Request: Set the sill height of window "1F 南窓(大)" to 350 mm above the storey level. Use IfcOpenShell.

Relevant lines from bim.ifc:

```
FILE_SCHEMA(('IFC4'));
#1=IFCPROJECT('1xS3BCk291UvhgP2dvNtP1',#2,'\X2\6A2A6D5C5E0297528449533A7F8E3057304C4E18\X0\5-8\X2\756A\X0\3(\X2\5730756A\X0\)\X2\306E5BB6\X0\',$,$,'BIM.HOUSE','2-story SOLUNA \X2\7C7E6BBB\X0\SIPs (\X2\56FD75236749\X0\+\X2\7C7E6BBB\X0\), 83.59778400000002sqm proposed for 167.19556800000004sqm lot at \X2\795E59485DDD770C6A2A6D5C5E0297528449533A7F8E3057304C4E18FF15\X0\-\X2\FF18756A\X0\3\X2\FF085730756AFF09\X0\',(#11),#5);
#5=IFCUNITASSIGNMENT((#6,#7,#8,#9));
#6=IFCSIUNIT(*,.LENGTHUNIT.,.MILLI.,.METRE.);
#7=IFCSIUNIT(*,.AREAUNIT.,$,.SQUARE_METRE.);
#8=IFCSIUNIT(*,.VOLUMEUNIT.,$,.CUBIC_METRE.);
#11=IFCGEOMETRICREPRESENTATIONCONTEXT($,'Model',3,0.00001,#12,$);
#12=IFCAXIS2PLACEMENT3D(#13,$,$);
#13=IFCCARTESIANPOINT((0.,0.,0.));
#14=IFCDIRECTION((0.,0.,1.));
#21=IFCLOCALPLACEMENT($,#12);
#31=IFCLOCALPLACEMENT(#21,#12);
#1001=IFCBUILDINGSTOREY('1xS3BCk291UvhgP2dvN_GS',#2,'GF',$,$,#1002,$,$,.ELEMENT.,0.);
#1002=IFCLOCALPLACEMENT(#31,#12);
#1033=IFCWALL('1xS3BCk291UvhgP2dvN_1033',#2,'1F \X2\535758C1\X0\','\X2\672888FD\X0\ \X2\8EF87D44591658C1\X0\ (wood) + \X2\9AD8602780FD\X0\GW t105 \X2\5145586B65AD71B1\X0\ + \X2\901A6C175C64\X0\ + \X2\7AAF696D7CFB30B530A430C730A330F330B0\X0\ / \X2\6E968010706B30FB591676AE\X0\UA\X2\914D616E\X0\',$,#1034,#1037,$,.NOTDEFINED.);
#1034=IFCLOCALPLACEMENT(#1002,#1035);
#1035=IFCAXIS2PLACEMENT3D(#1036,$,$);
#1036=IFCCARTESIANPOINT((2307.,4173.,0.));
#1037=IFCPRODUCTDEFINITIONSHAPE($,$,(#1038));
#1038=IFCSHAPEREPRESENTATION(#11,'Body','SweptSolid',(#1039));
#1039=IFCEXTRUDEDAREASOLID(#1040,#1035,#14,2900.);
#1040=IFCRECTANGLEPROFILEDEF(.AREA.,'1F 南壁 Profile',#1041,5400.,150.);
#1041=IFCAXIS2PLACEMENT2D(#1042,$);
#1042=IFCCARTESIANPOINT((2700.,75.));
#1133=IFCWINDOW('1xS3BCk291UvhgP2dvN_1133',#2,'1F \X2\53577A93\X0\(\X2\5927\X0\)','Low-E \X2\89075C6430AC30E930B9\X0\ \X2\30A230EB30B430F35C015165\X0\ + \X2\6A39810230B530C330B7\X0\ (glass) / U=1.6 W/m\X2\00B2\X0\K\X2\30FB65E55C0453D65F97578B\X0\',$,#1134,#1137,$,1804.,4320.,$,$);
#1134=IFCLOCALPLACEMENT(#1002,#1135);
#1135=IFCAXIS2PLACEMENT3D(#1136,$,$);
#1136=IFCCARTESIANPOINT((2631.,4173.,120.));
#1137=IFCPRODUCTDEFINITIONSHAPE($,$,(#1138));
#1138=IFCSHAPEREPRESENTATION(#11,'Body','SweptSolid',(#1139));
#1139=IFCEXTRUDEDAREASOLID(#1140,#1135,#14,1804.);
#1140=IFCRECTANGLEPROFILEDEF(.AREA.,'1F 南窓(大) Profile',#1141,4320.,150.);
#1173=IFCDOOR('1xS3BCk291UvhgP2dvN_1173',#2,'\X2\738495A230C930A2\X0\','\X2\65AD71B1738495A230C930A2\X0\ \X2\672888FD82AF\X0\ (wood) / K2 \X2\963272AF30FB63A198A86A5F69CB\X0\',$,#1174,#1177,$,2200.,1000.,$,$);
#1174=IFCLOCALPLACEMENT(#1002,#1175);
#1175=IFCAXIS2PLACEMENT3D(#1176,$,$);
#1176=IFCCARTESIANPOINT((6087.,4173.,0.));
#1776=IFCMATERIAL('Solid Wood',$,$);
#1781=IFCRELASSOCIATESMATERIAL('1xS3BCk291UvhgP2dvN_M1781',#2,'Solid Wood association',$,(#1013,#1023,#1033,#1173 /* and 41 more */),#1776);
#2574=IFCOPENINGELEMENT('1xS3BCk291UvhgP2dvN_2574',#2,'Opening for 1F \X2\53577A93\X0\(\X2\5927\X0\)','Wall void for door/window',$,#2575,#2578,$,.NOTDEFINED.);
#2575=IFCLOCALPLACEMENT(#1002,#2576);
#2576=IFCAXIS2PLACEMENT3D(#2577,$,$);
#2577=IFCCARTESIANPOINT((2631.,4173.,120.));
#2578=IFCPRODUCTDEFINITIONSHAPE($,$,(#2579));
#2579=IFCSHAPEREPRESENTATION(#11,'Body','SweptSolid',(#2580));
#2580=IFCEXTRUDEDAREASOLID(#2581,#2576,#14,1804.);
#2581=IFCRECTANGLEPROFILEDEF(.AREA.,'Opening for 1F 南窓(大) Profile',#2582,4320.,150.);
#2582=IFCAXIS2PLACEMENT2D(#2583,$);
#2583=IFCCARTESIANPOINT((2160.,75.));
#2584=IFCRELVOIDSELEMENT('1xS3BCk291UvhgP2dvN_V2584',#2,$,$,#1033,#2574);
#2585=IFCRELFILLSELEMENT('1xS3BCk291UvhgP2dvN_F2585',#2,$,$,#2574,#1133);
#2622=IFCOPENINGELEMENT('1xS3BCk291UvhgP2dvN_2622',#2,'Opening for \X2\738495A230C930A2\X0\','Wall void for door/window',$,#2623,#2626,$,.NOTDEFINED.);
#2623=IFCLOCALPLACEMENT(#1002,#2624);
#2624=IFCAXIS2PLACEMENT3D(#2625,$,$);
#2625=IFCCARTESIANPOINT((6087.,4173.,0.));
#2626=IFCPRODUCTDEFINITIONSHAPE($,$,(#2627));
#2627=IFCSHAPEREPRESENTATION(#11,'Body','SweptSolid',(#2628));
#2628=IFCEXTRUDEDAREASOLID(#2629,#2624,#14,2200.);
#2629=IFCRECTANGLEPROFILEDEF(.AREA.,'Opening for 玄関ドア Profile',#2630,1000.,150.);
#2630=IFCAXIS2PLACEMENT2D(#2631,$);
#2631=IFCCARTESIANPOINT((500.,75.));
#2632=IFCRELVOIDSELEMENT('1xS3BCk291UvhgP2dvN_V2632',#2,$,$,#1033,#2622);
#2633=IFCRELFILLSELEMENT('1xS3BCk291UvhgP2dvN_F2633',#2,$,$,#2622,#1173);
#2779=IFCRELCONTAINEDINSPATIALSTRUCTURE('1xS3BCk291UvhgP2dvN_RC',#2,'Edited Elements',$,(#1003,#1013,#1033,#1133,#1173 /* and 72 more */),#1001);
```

```python
import numpy as np
import ifcopenshell
import ifcopenshell.api.geometry
import ifcopenshell.geom
import ifcopenshell.util.element
import ifcopenshell.util.placement
import ifcopenshell.util.shape
import ifcopenshell.util.unit

model = ifcopenshell.open("bim.ifc")
unit_scale = ifcopenshell.util.unit.calculate_unit_scale(model)

window = model.by_guid("1xS3BCk291UvhgP2dvN_1133")
opening = window.FillsVoids[0].RelatingOpeningElement
storey = ifcopenshell.util.element.get_container(window, ifc_class="IfcBuildingStorey")
level = ifcopenshell.util.placement.get_local_placement(storey.ObjectPlacement)[2, 3]

# The opening's origin need not be at the sill, so measure its lowest point.
shape = ifcopenshell.geom.create_shape(ifcopenshell.geom.settings(), opening)
bottom = ifcopenshell.util.shape.get_shape_bottom_elevation(shape, shape.geometry) / unit_scale
dz = level + 0.35 / unit_scale - bottom

shift = np.array([0.0, 0.0, dz])
# The window is not placed relative to its opening, so move both.
for product in (opening, window):
    matrix = ifcopenshell.util.placement.get_local_placement(product.ObjectPlacement)
    matrix[:3, 3] += shift
    ifcopenshell.api.geometry.edit_object_placement(model, product=product, matrix=matrix, is_si=False)

print(f"moved by {dz * unit_scale:+.3f} m")

model.write("bim_updated.ifc")
```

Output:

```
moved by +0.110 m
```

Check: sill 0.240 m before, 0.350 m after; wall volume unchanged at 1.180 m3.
